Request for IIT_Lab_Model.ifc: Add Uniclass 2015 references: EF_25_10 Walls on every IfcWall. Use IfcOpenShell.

First a look at what the model holds.

```python
import ifcopenshell

model = ifcopenshell.open("IIT_Lab_Model.ifc")
print(model.schema)
print("classifications:", [c.Name for c in model.by_type("IfcClassification")])
for ifc_class in ("IfcDoor", "IfcRoof", "IfcStair", "IfcWall", "IfcWindow"):
    print(ifc_class, len(model.by_type(ifc_class)))
```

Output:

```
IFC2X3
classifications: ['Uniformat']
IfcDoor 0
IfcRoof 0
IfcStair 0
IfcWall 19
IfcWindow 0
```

```python
import ifcopenshell
import ifcopenshell.api.classification

model = ifcopenshell.open("IIT_Lab_Model.ifc")

# IFC2X3 requires Source and Edition and has no link from the project to the system.
system = model.create_entity("IfcClassification", Source="NBS", Edition="2015", Name="Uniclass 2015")

codes = {
    "IfcWall": ("EF_25_10", "Walls"),
}
for ifc_class, (code, name) in codes.items():
    products = model.by_type(ifc_class)
    ifcopenshell.api.classification.add_reference(
        model, products=products, classification=system, identification=code, name=name
    )
    print(code, len(products))

model.write("IIT_Lab_Model_rev.ifc")
```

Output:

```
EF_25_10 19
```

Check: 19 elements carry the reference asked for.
